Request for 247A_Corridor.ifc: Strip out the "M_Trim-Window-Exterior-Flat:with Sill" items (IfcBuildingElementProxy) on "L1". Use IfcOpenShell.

First a look at what the model holds.

```python
import ifcopenshell
import ifcopenshell.util.element

model = ifcopenshell.open("247A_Corridor.ifc")
print(model.schema)
storey = next(s for s in model.by_type("IfcBuildingStorey") if s.Name == "L1")
proxies = [e for e in ifcopenshell.util.element.get_decomposition(storey) if e.is_a("IfcBuildingElementProxy")]
seen = {}
for e in proxies:
    element_type = ifcopenshell.util.element.get_type(e)
    name = element_type.Name if element_type not in (None, e) else None
    seen[name] = seen.get(name, 0) + 1
for name, count in sorted(seen.items(), key=str):
    print(count, "x", name)
```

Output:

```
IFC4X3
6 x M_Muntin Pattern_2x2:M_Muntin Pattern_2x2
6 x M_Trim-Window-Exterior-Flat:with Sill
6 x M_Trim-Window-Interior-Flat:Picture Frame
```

```python
import ifcopenshell
import ifcopenshell.api.root
import ifcopenshell.util.element

model = ifcopenshell.open("247A_Corridor.ifc")

storey = next(s for s in model.by_type("IfcBuildingStorey") if s.Name == "L1")
proxies = [e for e in ifcopenshell.util.element.get_decomposition(storey) if e.is_a("IfcBuildingElementProxy")]
targets = [e for e in proxies if (t := ifcopenshell.util.element.get_type(e)) not in (None, e) and t.Name == "M_Trim-Window-Exterior-Flat:with Sill"]

for e in targets:
    ifcopenshell.api.root.remove_product(model, product=e)
print(len(targets), "removed")

model.write("247A_Corridor_edited.ifc")
```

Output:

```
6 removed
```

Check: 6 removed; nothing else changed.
